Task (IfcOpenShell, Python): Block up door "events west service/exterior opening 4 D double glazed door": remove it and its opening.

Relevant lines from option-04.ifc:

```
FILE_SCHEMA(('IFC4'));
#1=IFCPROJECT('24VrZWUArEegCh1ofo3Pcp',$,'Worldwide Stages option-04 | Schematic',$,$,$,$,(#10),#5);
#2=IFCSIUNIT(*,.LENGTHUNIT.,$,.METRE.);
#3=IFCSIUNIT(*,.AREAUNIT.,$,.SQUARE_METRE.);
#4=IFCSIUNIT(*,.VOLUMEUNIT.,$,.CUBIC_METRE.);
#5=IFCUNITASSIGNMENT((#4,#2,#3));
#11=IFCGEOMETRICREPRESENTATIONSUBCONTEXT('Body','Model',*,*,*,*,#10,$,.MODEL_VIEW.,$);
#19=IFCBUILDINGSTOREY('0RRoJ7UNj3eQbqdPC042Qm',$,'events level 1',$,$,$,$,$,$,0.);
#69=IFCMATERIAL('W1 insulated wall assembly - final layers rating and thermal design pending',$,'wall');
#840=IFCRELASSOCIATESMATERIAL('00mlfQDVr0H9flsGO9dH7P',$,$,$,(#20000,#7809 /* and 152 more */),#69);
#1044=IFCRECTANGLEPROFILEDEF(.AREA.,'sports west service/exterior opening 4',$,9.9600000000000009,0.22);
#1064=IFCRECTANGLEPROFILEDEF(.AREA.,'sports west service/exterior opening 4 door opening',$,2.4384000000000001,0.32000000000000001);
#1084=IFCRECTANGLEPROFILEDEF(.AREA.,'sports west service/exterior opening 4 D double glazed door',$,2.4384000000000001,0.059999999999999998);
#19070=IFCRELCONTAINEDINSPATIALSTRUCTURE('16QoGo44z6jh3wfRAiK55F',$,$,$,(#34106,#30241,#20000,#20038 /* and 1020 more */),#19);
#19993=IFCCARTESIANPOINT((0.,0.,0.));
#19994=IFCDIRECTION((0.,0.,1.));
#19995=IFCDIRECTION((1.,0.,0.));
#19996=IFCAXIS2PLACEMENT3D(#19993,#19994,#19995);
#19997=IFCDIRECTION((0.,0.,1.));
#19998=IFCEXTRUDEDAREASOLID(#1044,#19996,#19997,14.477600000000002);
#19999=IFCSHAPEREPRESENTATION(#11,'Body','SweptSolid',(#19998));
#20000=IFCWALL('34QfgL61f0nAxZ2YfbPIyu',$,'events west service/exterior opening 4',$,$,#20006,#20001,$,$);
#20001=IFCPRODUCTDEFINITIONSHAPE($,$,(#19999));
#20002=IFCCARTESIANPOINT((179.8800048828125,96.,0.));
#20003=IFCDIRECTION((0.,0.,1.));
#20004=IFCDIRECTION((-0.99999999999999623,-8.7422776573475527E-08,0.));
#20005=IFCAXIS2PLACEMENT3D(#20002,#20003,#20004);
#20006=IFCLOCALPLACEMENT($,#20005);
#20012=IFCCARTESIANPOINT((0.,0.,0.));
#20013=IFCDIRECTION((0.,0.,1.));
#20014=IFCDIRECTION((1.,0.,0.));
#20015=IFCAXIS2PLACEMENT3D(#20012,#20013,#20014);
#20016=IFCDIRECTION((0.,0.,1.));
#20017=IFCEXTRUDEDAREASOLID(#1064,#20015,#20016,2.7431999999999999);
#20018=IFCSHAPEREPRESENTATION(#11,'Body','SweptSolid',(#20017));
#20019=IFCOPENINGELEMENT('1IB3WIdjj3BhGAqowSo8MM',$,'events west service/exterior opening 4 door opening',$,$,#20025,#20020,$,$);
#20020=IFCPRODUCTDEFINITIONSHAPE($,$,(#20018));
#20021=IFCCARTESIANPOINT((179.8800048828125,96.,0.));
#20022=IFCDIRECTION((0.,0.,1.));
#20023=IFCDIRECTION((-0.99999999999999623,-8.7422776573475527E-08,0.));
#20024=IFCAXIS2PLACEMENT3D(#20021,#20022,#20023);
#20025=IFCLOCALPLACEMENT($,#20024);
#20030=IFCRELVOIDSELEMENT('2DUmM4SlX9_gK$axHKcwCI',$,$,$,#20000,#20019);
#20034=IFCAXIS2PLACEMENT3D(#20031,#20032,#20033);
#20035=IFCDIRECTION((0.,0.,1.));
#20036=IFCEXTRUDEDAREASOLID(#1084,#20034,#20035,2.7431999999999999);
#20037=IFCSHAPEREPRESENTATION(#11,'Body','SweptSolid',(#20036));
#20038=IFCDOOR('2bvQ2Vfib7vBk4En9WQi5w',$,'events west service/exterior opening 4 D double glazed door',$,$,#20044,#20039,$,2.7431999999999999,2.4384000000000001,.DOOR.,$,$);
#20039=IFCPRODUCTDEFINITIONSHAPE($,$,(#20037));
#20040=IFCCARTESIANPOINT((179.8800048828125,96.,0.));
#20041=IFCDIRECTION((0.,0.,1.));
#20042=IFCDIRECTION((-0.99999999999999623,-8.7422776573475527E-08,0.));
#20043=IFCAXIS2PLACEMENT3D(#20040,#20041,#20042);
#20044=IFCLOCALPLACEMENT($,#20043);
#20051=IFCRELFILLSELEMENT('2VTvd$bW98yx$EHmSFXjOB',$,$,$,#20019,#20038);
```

```python
import ifcopenshell
import ifcopenshell.api.feature
import ifcopenshell.api.root
import ifcopenshell.geom
import ifcopenshell.util.shape

model = ifcopenshell.open("option-04.ifc")
settings = ifcopenshell.geom.settings()


def volume(element):
    """Net volume in cubic metres, openings subtracted."""
    shape = ifcopenshell.geom.create_shape(settings, element)
    return ifcopenshell.util.shape.get_volume(shape.geometry)


door = model.by_guid("2bvQ2Vfib7vBk4En9WQi5w")
opening = door.FillsVoids[0].RelatingOpeningElement
wall = opening.VoidsElements[0].RelatingBuildingElement
before = volume(wall)

ifcopenshell.api.root.remove_product(model, product=door)
ifcopenshell.api.feature.remove_feature(model, feature=opening)

after = volume(wall)

print(f"wall volume {before:.3f} -> {after:.3f} m3")

model.write("option-04_v2.ifc")
```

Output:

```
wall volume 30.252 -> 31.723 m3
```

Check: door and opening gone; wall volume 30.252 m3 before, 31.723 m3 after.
